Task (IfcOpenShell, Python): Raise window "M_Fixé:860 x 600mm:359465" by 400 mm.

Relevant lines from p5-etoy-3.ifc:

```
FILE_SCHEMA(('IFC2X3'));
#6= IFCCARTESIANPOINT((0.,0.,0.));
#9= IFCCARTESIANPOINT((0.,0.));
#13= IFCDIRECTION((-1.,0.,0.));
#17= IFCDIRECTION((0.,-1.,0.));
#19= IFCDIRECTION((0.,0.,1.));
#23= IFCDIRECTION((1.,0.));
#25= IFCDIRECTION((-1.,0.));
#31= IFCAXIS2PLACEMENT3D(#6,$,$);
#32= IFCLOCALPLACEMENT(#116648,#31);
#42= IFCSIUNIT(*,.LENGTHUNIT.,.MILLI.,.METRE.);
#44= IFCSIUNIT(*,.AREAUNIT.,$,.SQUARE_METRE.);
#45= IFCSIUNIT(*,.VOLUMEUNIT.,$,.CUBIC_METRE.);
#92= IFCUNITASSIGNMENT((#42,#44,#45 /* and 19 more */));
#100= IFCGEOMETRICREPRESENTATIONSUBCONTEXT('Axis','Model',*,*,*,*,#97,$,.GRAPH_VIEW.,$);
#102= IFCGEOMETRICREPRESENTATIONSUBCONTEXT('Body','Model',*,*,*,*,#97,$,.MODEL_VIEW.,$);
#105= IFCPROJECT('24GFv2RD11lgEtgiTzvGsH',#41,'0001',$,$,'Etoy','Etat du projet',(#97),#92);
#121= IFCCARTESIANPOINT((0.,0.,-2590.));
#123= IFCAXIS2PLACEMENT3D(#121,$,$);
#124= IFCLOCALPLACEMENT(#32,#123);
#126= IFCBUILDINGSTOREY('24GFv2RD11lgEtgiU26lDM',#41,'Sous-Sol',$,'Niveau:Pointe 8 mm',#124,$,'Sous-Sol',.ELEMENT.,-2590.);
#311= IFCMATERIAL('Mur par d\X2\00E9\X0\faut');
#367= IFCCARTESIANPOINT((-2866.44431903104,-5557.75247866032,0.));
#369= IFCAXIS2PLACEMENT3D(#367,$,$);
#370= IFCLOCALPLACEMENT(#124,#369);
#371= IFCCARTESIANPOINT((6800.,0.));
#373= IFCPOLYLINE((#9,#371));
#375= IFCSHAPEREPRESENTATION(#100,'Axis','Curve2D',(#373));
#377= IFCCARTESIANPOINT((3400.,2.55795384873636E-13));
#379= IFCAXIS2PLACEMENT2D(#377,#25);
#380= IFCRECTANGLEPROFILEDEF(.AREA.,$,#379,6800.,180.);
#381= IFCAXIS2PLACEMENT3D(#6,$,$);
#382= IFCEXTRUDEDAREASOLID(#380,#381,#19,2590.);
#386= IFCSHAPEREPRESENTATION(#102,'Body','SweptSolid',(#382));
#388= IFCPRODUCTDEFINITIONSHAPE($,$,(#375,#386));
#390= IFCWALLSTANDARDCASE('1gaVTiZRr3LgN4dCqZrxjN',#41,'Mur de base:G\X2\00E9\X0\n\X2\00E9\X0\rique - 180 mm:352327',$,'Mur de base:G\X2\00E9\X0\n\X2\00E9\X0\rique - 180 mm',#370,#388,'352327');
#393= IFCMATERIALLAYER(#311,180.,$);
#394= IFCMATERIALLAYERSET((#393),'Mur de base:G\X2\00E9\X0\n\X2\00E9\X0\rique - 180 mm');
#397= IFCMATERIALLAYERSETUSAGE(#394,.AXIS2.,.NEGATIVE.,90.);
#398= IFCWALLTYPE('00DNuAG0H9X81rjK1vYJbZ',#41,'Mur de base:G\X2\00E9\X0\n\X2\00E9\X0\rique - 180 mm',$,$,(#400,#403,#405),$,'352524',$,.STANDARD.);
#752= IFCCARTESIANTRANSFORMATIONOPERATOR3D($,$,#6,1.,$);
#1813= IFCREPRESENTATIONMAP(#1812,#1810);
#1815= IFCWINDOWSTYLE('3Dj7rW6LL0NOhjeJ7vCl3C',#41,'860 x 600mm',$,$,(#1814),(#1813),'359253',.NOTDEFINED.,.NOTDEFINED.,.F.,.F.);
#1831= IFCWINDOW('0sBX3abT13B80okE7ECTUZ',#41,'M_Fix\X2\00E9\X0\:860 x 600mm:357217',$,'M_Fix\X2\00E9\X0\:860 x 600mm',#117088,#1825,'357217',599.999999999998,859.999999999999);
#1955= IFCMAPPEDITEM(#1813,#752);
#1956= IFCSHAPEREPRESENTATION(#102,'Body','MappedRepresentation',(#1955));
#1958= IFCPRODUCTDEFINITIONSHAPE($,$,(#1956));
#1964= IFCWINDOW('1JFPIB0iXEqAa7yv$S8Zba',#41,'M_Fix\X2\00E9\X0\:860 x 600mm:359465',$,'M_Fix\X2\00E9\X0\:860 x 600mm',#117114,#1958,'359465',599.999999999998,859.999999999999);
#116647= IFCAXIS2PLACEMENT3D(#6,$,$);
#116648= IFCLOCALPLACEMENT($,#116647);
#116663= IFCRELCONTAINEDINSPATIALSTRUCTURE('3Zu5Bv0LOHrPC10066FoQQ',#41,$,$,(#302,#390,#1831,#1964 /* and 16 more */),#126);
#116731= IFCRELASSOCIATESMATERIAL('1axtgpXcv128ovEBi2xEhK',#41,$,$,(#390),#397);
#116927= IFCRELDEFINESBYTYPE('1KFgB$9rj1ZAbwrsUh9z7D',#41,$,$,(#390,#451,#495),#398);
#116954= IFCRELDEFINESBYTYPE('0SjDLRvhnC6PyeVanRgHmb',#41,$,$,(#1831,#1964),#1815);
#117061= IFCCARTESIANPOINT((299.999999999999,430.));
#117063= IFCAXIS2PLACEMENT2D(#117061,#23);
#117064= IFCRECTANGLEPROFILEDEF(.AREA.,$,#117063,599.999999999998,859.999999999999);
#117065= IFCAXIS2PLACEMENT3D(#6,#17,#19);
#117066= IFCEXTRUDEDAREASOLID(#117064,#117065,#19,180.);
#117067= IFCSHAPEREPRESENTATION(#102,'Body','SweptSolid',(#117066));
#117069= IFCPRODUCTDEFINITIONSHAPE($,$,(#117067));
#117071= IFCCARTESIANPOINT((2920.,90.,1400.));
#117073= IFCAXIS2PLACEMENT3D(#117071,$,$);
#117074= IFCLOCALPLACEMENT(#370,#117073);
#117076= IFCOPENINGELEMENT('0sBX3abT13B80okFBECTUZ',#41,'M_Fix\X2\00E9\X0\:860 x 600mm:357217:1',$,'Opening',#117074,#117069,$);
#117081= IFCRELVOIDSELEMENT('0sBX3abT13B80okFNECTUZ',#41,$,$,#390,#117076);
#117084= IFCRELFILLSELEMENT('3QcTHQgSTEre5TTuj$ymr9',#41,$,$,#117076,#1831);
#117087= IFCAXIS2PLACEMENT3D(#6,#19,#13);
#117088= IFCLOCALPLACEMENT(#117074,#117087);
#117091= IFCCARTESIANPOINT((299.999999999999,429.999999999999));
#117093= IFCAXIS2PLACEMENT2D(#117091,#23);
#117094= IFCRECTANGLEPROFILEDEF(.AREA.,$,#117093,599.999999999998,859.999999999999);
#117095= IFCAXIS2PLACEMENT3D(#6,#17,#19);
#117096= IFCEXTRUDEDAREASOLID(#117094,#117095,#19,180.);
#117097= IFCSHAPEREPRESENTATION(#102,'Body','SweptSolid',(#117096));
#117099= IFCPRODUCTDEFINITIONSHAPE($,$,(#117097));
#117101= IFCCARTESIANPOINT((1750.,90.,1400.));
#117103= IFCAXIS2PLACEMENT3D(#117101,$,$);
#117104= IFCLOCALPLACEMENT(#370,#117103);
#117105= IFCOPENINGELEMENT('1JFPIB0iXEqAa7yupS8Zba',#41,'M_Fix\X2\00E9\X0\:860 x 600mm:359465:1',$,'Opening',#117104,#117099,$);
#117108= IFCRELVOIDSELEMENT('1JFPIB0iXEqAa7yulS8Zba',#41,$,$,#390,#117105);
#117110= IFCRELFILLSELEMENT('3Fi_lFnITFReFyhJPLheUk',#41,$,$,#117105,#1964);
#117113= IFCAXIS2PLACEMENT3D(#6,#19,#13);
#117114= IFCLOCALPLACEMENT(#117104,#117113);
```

```python
import numpy as np
import ifcopenshell
import ifcopenshell.api.geometry
import ifcopenshell.util.placement
import ifcopenshell.util.unit

model = ifcopenshell.open("p5-etoy-3.ifc")
unit_scale = ifcopenshell.util.unit.calculate_unit_scale(model)

window = model.by_guid("1JFPIB0iXEqAa7yv$S8Zba")
opening = window.FillsVoids[0].RelatingOpeningElement
dz = 0.4 / unit_scale

shift = np.array([0.0, 0.0, dz])
# The window is placed relative to its opening, so it follows when the opening moves.
matrix = ifcopenshell.util.placement.get_local_placement(opening.ObjectPlacement)
matrix[:3, 3] += shift
ifcopenshell.api.geometry.edit_object_placement(
    model, product=opening, matrix=matrix, is_si=False, should_transform_children=True
)

print(f"moved by {dz * unit_scale:+.3f} m")

model.write("p5-etoy-3_updated.ifc")
```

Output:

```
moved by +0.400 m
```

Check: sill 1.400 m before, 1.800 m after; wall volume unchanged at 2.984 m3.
